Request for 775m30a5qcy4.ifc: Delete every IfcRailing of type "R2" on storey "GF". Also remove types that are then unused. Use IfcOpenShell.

First a look at what the model holds.

```python
import ifcopenshell
import ifcopenshell.util.element

model = ifcopenshell.open("775m30a5qcy4.ifc")
print(model.schema)
storey = next(s for s in model.by_type("IfcBuildingStorey") if s.Name == "GF")
railings = [e for e in ifcopenshell.util.element.get_decomposition(storey) if e.is_a("IfcRailing")]
seen = {}
for e in railings:
    element_type = ifcopenshell.util.element.get_type(e)
    name = element_type.Name if element_type not in (None, e) else None
    seen[name] = seen.get(name, 0) + 1
for name, count in sorted(seen.items(), key=str):
    print(count, "x", name)
```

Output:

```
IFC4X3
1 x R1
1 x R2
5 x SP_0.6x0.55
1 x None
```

```python
import ifcopenshell
import ifcopenshell.api.root
import ifcopenshell.util.element

model = ifcopenshell.open("775m30a5qcy4.ifc")

storey = next(s for s in model.by_type("IfcBuildingStorey") if s.Name == "GF")
railings = [e for e in ifcopenshell.util.element.get_decomposition(storey) if e.is_a("IfcRailing")]
targets = [e for e in railings if (t := ifcopenshell.util.element.get_type(e)) not in (None, e) and t.Name == "R2"]
types = {ifcopenshell.util.element.get_type(e) for e in targets} - {None, *targets}

for e in targets:
    ifcopenshell.api.root.remove_product(model, product=e)
print(len(targets), "removed")

unused = [t for t in types if not ifcopenshell.util.element.get_types(t)]
for t in unused:
    ifcopenshell.api.root.remove_product(model, product=t)
print(len(unused), "unused types removed")

model.write("775m30a5qcy4_edited.ifc")
```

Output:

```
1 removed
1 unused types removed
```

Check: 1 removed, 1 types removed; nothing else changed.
